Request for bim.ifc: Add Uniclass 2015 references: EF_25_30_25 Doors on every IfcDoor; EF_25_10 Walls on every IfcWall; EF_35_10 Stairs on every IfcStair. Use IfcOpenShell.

First a look at what the model holds.

```python
import ifcopenshell

model = ifcopenshell.open("bim.ifc")
print(model.schema)
print("classifications:", [c.Name for c in model.by_type("IfcClassification")])
for ifc_class in ("IfcDoor", "IfcRoof", "IfcStair", "IfcWall", "IfcWindow"):
    print(ifc_class, len(model.by_type(ifc_class)))
```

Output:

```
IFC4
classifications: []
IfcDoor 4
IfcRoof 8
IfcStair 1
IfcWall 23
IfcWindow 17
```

```python
import ifcopenshell
import ifcopenshell.api.classification

model = ifcopenshell.open("bim.ifc")

system = ifcopenshell.api.classification.add_classification(model, classification="Uniclass 2015")

codes = {
    "IfcDoor": ("EF_25_30_25", "Doors"),
    "IfcWall": ("EF_25_10", "Walls"),
    "IfcStair": ("EF_35_10", "Stairs"),
}
for ifc_class, (code, name) in codes.items():
    products = model.by_type(ifc_class)
    ifcopenshell.api.classification.add_reference(
        model, products=products, classification=system, identification=code, name=name
    )
    print(code, len(products))

model.write("bim_v2.ifc")
```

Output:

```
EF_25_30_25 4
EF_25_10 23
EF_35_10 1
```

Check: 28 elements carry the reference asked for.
